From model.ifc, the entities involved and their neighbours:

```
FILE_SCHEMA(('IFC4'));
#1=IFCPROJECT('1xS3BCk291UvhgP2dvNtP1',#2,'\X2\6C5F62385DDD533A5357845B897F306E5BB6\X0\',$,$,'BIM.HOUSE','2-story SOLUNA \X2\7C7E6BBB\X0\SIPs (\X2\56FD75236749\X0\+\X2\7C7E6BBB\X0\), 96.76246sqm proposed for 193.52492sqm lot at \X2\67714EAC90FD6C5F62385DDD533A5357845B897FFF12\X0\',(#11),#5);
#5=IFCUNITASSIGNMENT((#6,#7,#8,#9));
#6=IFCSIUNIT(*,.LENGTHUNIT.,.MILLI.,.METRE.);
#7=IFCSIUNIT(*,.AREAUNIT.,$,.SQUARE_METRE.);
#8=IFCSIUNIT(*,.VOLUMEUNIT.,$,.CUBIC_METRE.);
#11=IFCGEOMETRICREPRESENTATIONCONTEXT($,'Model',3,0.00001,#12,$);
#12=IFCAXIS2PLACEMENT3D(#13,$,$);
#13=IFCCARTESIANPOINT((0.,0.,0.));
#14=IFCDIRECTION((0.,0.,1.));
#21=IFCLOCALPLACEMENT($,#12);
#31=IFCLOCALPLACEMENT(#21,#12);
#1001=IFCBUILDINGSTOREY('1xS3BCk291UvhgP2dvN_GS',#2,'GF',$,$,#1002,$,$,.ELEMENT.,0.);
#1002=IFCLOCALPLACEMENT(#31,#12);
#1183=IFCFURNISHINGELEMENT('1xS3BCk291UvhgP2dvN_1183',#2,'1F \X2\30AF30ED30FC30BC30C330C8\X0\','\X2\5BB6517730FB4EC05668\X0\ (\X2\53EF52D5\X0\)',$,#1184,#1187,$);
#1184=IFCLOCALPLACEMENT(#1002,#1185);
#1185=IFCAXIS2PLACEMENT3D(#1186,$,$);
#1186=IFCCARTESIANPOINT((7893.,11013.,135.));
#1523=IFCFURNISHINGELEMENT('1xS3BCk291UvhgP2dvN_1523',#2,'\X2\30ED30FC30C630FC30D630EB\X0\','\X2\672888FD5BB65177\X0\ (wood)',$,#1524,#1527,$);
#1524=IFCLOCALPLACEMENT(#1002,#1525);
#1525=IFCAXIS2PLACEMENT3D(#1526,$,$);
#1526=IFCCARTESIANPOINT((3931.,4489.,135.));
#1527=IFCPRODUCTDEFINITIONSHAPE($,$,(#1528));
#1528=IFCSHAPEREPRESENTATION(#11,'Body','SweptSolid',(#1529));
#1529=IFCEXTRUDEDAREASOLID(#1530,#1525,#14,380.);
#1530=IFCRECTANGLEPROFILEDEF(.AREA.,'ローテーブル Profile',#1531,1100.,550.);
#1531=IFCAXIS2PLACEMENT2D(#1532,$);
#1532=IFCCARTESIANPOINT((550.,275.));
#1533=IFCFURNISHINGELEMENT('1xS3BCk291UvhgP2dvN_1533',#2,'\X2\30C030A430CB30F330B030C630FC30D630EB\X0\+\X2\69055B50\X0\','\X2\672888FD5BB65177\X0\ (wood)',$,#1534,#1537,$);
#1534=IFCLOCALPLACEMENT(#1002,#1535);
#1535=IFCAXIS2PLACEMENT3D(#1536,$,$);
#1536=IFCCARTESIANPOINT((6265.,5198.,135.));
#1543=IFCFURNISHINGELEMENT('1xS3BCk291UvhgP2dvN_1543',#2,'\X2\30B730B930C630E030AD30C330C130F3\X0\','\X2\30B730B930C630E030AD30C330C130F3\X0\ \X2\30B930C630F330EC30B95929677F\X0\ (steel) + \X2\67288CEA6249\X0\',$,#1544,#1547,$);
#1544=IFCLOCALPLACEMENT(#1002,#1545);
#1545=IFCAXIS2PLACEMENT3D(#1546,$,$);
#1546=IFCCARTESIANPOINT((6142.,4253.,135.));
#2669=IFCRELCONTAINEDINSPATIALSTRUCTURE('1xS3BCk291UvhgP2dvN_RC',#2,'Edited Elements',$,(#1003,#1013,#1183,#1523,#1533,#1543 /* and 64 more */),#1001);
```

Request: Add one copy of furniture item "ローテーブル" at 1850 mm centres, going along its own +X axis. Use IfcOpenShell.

```python
import ifcopenshell
import ifcopenshell.api.geometry
import ifcopenshell.api.root
import ifcopenshell.util.element
import ifcopenshell.util.placement

model = ifcopenshell.open("model.ifc")


def reuse_history(source, copy):
    """copy_class also copies each property set's owner history, people and application; keep the originals."""
    for rel in copy.IsDefinedBy:
        if rel.is_a("IfcRelDefinesByProperties") and (history := rel.RelatingPropertyDefinition.OwnerHistory):
            rel.RelatingPropertyDefinition.OwnerHistory = source.OwnerHistory
            ifcopenshell.util.element.remove_deep2(model, history)


source = model.by_id(1523)
base = ifcopenshell.util.placement.get_local_placement(source.ObjectPlacement)
step = base[:3, 0] * 1850.0

for i in range(1, 2):
    copy = ifcopenshell.api.root.copy_class(model, product=source)
    copy.Representation = ifcopenshell.util.element.copy_deep(
        model, source.Representation, exclude=["IfcGeometricRepresentationContext", "IfcRepresentationMap"]
    )
    reuse_history(source, copy)
    matrix = base.copy()
    matrix[:3, 3] += i * step
    print("added at", matrix[:3, 3].round(3) + 0.0)
    ifcopenshell.api.geometry.edit_object_placement(model, product=copy, matrix=matrix, is_si=False)

model.write("model_edited.ifc")
```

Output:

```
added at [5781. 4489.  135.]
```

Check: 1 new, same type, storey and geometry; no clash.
